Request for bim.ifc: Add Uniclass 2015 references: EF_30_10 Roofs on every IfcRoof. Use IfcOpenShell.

First a look at what the model holds.

```python
import ifcopenshell

model = ifcopenshell.open("bim.ifc")
print(model.schema)
print("classifications:", [c.Name for c in model.by_type("IfcClassification")])
for ifc_class in ("IfcDoor", "IfcRoof", "IfcStair", "IfcWall", "IfcWindow"):
    print(ifc_class, len(model.by_type(ifc_class)))
```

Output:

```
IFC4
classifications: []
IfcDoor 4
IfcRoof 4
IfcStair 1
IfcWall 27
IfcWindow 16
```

```python
import ifcopenshell
import ifcopenshell.api.classification

model = ifcopenshell.open("bim.ifc")

system = ifcopenshell.api.classification.add_classification(model, classification="Uniclass 2015")

codes = {
    "IfcRoof": ("EF_30_10", "Roofs"),
}
for ifc_class, (code, name) in codes.items():
    products = model.by_type(ifc_class)
    ifcopenshell.api.classification.add_reference(
        model, products=products, classification=system, identification=code, name=name
    )
    print(code, len(products))

model.write("bim_rev.ifc")
```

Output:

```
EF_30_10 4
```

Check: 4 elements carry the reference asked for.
